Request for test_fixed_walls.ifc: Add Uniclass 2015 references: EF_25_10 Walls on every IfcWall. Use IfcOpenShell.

First a look at what the model holds.

```python
import ifcopenshell

model = ifcopenshell.open("test_fixed_walls.ifc")
print(model.schema)
print("classifications:", [c.Name for c in model.by_type("IfcClassification")])
for ifc_class in ("IfcDoor", "IfcRoof", "IfcStair", "IfcWall", "IfcWindow"):
    print(ifc_class, len(model.by_type(ifc_class)))
```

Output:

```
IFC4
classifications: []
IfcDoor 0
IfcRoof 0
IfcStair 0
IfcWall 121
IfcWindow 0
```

```python
import ifcopenshell
import ifcopenshell.api.classification

model = ifcopenshell.open("test_fixed_walls.ifc")

system = ifcopenshell.api.classification.add_classification(model, classification="Uniclass 2015")

codes = {
    "IfcWall": ("EF_25_10", "Walls"),
}
for ifc_class, (code, name) in codes.items():
    products = model.by_type(ifc_class)
    ifcopenshell.api.classification.add_reference(
        model, products=products, classification=system, identification=code, name=name
    )
    print(code, len(products))

model.write("test_fixed_walls_edited.ifc")
```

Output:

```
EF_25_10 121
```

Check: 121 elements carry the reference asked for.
